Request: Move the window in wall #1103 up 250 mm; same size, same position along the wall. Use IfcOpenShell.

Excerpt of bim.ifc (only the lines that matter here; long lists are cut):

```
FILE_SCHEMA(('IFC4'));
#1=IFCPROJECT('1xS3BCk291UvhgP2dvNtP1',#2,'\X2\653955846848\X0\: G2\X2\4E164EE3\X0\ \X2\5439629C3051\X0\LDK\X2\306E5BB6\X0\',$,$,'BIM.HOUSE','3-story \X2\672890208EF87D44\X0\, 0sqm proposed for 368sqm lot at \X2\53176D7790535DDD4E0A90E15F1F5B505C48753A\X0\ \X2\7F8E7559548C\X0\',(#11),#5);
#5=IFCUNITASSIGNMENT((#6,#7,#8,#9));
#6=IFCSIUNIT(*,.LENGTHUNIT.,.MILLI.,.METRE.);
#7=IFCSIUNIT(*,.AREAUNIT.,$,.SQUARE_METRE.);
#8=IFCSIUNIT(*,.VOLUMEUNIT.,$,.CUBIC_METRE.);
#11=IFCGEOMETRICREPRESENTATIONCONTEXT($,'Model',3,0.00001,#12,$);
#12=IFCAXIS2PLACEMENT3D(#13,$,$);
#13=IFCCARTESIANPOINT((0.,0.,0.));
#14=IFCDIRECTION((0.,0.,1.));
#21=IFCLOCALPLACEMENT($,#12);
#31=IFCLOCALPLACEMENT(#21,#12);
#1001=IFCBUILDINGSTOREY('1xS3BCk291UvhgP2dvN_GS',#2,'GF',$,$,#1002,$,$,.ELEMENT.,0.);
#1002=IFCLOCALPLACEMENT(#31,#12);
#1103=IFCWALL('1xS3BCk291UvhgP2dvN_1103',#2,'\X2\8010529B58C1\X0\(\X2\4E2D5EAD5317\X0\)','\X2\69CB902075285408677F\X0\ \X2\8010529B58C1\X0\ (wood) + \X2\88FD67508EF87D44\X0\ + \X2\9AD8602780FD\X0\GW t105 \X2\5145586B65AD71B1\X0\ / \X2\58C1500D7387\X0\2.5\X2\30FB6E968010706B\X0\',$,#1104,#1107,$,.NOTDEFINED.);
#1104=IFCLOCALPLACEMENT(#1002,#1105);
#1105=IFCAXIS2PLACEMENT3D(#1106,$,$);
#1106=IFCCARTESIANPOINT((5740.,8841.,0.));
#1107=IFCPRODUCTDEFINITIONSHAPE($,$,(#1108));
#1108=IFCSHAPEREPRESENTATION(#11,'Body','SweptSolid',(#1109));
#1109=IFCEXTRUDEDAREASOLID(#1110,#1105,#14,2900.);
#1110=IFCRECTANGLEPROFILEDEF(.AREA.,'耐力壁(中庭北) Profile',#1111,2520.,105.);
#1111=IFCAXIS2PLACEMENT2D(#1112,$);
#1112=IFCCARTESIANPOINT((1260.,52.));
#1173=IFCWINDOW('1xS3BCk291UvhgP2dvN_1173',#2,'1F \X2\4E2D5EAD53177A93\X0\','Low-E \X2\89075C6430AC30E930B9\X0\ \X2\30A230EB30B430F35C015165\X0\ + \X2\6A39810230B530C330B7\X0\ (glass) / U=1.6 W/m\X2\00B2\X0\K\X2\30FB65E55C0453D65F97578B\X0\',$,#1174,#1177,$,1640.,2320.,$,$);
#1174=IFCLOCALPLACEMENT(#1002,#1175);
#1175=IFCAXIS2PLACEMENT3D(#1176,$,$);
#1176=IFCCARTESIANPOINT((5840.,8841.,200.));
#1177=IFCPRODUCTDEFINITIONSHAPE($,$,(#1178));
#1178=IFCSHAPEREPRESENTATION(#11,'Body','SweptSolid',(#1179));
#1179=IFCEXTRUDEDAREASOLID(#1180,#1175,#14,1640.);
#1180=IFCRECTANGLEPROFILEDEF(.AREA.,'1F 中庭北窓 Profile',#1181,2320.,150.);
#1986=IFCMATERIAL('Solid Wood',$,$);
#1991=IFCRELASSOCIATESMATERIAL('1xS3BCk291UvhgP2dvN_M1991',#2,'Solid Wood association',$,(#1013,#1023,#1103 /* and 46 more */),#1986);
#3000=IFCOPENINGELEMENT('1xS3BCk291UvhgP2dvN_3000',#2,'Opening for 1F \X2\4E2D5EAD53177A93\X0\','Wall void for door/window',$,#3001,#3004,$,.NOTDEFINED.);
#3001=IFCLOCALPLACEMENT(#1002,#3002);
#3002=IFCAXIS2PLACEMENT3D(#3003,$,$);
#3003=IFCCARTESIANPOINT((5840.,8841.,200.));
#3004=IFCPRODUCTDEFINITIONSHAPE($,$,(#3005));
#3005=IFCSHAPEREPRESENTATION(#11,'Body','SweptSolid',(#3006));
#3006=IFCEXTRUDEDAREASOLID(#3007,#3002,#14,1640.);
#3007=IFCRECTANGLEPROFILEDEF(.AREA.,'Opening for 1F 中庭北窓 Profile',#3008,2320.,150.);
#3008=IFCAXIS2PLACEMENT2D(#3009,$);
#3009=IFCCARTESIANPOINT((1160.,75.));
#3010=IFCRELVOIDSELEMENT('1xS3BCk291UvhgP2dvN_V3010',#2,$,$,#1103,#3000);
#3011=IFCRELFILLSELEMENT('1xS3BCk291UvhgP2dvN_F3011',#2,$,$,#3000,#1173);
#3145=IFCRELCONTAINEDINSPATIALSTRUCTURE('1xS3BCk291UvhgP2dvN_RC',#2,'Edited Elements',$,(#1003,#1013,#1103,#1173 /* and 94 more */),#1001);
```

```python
import numpy as np
import ifcopenshell
import ifcopenshell.api.geometry
import ifcopenshell.util.placement
import ifcopenshell.util.unit

model = ifcopenshell.open("bim.ifc")
unit_scale = ifcopenshell.util.unit.calculate_unit_scale(model)

window = model.by_guid("1xS3BCk291UvhgP2dvN_1173")
opening = window.FillsVoids[0].RelatingOpeningElement
dz = 250.0

shift = np.array([0.0, 0.0, dz])
# The window is not placed relative to its opening, so move both.
for product in (opening, window):
    matrix = ifcopenshell.util.placement.get_local_placement(product.ObjectPlacement)
    matrix[:3, 3] += shift
    ifcopenshell.api.geometry.edit_object_placement(model, product=product, matrix=matrix, is_si=False)

print(f"moved by {dz * unit_scale:+.3f} m")

model.write("bim_updated.ifc")
```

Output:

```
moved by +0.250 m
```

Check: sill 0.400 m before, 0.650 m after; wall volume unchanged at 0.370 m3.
